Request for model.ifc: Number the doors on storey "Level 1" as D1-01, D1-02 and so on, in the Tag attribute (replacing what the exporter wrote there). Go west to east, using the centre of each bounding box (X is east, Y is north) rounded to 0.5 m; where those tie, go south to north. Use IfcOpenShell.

First a look at what the model holds.

```python
import ifcopenshell
import ifcopenshell.util.element
import ifcopenshell.util.placement

model = ifcopenshell.open("model.ifc")
print(model.schema)
storey = next(s for s in model.by_type("IfcBuildingStorey") if s.Name == "Level 1")
doors = [e for e in ifcopenshell.util.element.get_decomposition(storey) if e.is_a("IfcDoor")]
for e in sorted(doors, key=lambda e: e.id()):
    origin = ifcopenshell.util.placement.get_local_placement(e.ObjectPlacement)[:3, 3]
    print(e.id(), e.Tag, e.Name, origin.round(2) + 0.0, sep=" | ")
```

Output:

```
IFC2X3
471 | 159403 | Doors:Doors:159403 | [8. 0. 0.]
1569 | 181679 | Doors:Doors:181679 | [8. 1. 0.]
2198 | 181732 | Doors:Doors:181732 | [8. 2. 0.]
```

```python
import ifcopenshell
import ifcopenshell.geom
import ifcopenshell.util.element
import ifcopenshell.util.shape

model = ifcopenshell.open("model.ifc")
settings = ifcopenshell.geom.settings()
settings.set("use-world-coords", True)


def centre(element):
    shape = ifcopenshell.geom.create_shape(settings, element)
    return ifcopenshell.util.shape.get_bbox_centroid(shape.geometry)


storey = next(s for s in model.by_type("IfcBuildingStorey") if s.Name == "Level 1")
doors = [e for e in ifcopenshell.util.element.get_decomposition(storey) if e.is_a("IfcDoor")]

# Insertion points can sit at a corner or the storey origin, so sort by the geometry (in metres).
centres = {e: centre(e) for e in doors}
doors.sort(key=lambda e: (round(centres[e][0] / 0.5), centres[e][1]))

for i, e in enumerate(doors, start=1):
    number = f"D1-{i:02d}"
    e.Tag = number
    print(e.id(), number)

model.write("model_rev.ifc")
```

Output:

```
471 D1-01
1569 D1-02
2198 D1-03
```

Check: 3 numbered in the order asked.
